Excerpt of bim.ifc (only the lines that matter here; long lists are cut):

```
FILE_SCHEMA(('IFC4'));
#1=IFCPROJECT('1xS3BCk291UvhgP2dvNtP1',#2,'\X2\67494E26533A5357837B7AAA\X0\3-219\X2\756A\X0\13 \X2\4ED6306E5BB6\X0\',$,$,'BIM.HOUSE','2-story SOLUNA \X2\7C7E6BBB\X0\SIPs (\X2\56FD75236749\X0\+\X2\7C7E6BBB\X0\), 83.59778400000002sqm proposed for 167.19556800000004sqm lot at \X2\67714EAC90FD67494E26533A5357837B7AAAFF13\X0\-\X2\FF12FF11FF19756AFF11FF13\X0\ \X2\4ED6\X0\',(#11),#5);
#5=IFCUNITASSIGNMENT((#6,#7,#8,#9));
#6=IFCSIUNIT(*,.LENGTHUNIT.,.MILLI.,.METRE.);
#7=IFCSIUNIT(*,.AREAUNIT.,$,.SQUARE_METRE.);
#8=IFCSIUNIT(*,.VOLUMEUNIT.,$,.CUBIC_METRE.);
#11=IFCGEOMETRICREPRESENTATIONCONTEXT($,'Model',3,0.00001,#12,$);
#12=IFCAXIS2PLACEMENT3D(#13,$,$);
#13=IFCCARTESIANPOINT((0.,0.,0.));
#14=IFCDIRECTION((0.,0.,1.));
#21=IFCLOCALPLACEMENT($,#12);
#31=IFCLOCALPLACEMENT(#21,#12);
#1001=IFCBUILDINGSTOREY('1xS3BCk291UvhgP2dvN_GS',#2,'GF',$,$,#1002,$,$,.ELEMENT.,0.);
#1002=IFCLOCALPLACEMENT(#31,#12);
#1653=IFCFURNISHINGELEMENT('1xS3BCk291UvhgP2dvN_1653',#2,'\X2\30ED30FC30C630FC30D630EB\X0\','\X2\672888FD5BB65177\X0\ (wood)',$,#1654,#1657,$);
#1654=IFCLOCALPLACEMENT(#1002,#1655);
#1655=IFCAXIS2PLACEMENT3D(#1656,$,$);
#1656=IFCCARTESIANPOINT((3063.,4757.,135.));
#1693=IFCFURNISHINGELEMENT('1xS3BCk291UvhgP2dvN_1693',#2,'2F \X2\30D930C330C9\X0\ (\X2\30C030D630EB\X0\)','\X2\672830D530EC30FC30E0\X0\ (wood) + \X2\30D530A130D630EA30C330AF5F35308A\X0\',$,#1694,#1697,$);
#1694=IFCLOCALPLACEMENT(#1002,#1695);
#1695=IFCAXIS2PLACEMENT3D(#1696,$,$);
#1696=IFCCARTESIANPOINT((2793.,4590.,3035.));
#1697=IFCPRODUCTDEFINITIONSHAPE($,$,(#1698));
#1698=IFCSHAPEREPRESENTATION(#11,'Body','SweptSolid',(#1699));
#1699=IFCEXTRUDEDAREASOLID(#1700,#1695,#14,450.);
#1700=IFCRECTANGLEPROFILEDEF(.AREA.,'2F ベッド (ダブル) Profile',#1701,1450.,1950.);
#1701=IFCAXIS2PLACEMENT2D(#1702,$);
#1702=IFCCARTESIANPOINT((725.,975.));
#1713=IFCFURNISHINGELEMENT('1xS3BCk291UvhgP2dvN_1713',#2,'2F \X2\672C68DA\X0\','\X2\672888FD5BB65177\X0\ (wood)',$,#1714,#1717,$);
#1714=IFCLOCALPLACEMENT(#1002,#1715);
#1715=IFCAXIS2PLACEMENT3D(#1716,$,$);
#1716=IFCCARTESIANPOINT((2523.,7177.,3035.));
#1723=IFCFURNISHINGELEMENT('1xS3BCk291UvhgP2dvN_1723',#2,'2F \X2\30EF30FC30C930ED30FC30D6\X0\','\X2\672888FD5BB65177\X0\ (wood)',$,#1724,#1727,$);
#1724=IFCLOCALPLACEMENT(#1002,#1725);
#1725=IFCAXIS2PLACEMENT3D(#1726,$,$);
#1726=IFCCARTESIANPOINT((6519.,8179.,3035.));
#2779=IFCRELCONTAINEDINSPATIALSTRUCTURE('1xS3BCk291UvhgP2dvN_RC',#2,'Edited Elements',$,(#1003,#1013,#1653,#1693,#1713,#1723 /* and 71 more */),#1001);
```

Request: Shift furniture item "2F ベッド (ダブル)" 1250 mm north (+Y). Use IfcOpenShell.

```python
import ifcopenshell
import ifcopenshell.api.geometry
import ifcopenshell.util.placement
import ifcopenshell.util.unit

model = ifcopenshell.open("bim.ifc")
unit_scale = ifcopenshell.util.unit.calculate_unit_scale(model)

item = model.by_guid("1xS3BCk291UvhgP2dvN_1693")
matrix = ifcopenshell.util.placement.get_local_placement(item.ObjectPlacement)
matrix[1, 3] += 1.25 / unit_scale
ifcopenshell.api.geometry.edit_object_placement(model, product=item, matrix=matrix, is_si=False)

print(ifcopenshell.util.placement.get_local_placement(item.ObjectPlacement).round(3) + 0.0)

model.write("bim_rev.ifc")
```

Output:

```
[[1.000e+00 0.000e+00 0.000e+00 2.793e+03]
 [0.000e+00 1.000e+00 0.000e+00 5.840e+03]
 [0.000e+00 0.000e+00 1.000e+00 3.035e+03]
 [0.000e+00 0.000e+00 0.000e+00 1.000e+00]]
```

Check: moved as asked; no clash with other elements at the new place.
